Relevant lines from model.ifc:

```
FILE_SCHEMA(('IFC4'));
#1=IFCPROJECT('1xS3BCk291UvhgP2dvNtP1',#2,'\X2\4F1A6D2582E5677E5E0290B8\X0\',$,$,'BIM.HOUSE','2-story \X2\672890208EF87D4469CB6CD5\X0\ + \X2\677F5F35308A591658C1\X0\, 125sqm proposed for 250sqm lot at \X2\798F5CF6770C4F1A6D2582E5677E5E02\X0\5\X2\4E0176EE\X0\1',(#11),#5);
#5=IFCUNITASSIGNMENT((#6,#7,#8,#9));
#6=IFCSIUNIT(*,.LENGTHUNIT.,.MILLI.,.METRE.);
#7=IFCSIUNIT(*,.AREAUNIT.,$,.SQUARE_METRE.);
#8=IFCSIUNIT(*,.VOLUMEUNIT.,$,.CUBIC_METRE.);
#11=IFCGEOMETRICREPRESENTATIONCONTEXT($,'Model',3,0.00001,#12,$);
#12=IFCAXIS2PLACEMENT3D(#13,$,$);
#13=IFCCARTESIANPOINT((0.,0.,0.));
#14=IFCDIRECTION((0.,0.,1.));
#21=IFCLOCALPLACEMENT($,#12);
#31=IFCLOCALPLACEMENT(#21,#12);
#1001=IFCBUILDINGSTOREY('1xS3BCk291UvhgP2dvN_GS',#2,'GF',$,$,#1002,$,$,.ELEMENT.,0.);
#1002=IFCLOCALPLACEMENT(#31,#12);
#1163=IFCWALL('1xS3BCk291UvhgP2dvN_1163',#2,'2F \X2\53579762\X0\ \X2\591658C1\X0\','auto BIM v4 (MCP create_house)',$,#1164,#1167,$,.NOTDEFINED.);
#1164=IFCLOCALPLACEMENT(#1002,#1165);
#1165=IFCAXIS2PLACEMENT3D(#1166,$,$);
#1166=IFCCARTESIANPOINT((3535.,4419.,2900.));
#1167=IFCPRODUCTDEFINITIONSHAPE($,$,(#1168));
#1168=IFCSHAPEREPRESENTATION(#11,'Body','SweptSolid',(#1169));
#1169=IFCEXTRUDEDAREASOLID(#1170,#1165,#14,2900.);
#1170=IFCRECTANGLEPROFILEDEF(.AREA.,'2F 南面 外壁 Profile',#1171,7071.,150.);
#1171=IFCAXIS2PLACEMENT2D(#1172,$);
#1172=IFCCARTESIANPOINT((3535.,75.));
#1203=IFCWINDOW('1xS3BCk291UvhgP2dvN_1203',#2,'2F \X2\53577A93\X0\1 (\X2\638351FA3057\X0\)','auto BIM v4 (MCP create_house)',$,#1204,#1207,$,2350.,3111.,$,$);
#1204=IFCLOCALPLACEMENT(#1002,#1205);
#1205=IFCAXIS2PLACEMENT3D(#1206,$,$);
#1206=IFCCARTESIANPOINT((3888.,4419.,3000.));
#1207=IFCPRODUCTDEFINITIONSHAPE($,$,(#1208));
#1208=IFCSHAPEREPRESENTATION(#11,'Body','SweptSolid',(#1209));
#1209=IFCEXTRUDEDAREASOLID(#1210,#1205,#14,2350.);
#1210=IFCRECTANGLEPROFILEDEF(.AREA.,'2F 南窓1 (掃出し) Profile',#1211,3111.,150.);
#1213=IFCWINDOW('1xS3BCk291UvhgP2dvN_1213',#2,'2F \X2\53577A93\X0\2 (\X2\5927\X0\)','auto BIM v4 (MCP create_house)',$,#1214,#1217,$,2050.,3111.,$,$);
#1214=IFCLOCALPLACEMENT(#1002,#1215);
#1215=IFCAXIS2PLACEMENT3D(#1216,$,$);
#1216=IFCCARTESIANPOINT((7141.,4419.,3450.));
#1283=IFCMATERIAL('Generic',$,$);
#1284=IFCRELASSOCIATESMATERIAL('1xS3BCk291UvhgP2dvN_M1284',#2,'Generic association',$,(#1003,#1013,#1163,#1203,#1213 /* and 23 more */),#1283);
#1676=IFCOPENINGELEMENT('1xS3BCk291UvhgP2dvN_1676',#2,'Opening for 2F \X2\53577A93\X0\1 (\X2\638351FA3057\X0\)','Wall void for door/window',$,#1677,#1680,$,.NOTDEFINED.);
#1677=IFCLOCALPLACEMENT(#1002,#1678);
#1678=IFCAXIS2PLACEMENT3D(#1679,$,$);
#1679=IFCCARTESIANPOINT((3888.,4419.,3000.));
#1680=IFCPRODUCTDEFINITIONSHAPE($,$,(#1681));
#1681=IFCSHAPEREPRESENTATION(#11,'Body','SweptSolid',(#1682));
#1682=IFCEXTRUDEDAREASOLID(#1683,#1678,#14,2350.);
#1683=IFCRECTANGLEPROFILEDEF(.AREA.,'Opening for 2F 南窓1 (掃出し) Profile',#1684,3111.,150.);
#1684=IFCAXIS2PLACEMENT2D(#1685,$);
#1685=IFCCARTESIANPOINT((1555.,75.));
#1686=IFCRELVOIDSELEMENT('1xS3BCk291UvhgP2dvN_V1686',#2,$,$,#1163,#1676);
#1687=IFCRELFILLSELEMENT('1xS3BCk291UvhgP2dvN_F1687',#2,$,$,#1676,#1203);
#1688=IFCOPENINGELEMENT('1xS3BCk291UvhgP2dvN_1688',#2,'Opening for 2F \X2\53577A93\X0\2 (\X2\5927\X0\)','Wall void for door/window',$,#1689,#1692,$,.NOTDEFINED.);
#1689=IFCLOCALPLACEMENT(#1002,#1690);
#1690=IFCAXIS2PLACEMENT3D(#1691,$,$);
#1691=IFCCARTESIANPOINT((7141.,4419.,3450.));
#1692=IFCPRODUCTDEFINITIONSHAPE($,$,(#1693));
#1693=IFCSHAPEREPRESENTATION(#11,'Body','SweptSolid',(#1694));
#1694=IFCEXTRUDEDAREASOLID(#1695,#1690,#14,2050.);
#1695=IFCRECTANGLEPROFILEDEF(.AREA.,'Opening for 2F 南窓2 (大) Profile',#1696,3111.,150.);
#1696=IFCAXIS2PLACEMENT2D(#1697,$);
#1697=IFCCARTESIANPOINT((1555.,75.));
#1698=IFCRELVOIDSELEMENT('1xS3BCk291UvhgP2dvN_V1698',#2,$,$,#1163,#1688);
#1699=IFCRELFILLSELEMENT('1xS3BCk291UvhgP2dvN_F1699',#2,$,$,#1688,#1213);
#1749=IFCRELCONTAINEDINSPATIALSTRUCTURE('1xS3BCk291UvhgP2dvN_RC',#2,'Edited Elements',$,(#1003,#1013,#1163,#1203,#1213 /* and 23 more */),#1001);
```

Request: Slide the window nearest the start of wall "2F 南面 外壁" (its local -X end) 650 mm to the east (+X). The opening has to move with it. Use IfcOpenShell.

```python
import ifcopenshell
import ifcopenshell.api.geometry
import ifcopenshell.util.placement
import ifcopenshell.util.unit

model = ifcopenshell.open("model.ifc")
unit_scale = ifcopenshell.util.unit.calculate_unit_scale(model)

window = model.by_guid("1xS3BCk291UvhgP2dvN_1203")
opening = window.FillsVoids[0].RelatingOpeningElement
wall = opening.VoidsElements[0].RelatingBuildingElement

wall_matrix = ifcopenshell.util.placement.get_local_placement(wall.ObjectPlacement)
shift = wall_matrix[:3, 0] * 0.65 / unit_scale
before = ifcopenshell.util.placement.get_local_placement(window.ObjectPlacement)[:3, 3].copy()

# The window is not placed relative to its opening, so move both.
for product in (opening, window):
    matrix = ifcopenshell.util.placement.get_local_placement(product.ObjectPlacement)
    matrix[:3, 3] += shift
    ifcopenshell.api.geometry.edit_object_placement(model, product=product, matrix=matrix, is_si=False)

after = ifcopenshell.util.placement.get_local_placement(window.ObjectPlacement)[:3, 3]
print("window moved by", (after - before).round(3) + 0.0)

model.write("model-out.ifc")
```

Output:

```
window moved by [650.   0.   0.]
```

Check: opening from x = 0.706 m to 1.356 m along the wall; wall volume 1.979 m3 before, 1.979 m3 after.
